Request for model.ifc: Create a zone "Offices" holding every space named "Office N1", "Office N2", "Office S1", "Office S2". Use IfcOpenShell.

First a look at what the model holds.

```python
import ifcopenshell

model = ifcopenshell.open("model.ifc")
print(model.schema)
seen = {}
for space in model.by_type("IfcSpace"):
    seen[space.LongName] = seen.get(space.LongName, 0) + 1
for name, count in sorted(seen.items(), key=str):
    print(count, "x", name)
print("zones:", [z.Name for z in model.by_type("IfcZone")][:20])
```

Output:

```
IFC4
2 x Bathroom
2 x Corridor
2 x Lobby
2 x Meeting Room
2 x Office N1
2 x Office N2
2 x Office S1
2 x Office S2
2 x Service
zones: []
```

```python
import ifcopenshell
import ifcopenshell.api.group
import ifcopenshell.api.root

model = ifcopenshell.open("model.ifc")

names = {"Office N1", "Office N2", "Office S1", "Office S2"}
spaces = [s for s in model.by_type("IfcSpace") if s.LongName in names]

zone = ifcopenshell.api.root.create_entity(model, ifc_class="IfcZone", name="Offices")
ifcopenshell.api.group.assign_group(model, products=spaces, group=zone)
print(len(spaces), "spaces in", zone.Name)

model.write("model_edited.ifc")
```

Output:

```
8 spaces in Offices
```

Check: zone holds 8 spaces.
